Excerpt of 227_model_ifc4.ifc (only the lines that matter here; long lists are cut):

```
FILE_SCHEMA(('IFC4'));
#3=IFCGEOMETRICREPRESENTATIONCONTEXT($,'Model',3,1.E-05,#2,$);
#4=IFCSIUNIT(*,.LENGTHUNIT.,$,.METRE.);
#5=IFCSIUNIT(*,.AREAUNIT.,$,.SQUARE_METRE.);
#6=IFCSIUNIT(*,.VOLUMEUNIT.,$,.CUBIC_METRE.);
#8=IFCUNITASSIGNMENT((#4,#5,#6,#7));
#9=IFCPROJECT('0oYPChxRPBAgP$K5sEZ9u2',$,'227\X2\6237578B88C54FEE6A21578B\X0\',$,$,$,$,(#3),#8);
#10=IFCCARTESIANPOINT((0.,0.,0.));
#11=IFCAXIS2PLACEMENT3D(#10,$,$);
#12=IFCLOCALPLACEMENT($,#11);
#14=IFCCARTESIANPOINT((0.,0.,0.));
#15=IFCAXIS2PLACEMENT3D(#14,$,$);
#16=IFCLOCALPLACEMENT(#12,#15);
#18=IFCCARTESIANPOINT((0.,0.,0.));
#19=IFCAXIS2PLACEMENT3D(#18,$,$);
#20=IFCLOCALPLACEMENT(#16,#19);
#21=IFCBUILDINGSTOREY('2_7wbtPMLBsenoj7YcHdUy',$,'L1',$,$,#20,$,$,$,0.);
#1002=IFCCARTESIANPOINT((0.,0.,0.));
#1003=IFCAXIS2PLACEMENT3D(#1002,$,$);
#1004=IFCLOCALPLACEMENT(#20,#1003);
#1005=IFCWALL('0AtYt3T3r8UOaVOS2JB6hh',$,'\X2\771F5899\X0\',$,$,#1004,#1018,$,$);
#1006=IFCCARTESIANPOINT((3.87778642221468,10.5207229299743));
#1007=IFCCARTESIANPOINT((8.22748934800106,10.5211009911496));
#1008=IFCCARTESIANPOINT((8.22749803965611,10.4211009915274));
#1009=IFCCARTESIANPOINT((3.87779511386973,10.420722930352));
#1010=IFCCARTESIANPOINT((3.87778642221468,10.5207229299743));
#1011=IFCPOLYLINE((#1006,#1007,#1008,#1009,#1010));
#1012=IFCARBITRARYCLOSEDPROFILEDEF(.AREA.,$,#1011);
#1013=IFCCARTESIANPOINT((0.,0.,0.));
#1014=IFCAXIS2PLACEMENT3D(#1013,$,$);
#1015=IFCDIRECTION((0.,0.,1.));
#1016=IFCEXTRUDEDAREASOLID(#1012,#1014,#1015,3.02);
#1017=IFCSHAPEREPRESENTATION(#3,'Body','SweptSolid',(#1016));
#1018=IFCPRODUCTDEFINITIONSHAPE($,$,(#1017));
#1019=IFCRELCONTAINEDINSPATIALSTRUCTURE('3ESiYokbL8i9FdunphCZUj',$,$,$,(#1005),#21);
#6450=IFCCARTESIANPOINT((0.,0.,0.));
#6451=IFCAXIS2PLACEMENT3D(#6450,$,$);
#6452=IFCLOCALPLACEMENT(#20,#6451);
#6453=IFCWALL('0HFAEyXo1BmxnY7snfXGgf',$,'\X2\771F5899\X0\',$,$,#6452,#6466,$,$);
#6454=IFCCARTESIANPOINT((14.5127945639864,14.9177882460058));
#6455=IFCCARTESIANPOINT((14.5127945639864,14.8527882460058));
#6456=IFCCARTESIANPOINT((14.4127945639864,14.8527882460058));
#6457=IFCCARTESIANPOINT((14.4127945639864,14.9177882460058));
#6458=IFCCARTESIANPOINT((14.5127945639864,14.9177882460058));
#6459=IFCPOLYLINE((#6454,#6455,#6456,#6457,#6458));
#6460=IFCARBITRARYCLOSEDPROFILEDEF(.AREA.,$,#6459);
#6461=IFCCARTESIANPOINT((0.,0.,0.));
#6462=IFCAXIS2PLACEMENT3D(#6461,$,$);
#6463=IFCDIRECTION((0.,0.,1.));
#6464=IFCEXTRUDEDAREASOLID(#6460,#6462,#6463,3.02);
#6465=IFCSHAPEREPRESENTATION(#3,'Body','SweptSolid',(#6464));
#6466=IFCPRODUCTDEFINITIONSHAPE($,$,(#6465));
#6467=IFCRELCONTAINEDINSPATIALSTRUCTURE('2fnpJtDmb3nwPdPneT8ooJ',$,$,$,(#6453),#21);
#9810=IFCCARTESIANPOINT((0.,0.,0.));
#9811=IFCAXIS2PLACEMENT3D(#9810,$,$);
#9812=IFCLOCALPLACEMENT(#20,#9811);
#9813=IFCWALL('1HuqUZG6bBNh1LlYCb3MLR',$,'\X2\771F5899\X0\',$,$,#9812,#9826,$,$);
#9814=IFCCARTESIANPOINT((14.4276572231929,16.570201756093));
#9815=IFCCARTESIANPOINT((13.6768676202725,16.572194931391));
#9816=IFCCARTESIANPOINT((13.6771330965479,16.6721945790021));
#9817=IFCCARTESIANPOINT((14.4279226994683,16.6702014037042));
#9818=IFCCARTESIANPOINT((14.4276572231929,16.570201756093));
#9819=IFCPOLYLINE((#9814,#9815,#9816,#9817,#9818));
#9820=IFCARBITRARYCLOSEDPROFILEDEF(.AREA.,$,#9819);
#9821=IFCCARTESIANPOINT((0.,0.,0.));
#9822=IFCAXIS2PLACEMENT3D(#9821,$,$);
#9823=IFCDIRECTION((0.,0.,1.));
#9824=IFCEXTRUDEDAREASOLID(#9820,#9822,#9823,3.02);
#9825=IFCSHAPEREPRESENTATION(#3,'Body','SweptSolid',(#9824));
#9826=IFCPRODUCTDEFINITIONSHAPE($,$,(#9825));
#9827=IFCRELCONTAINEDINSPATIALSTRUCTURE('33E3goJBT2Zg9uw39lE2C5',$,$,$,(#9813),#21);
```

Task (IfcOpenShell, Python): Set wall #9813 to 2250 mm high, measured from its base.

```python
import ifcopenshell
import ifcopenshell.geom
import ifcopenshell.util.shape
import ifcopenshell.util.unit

model = ifcopenshell.open("227_model_ifc4.ifc")
unit_scale = ifcopenshell.util.unit.calculate_unit_scale(model)
settings = ifcopenshell.geom.settings()


def volume(element):
    """Net volume in cubic metres, openings subtracted."""
    shape = ifcopenshell.geom.create_shape(settings, element)
    return ifcopenshell.util.shape.get_volume(shape.geometry)


wall = model.by_guid("1HuqUZG6bBNh1LlYCb3MLR")
before = volume(wall)

body = next(r for r in wall.Representation.Representations if r.RepresentationIdentifier == "Body")
solid = body.Items[0]
old_height = solid.Depth
solid.Depth = 2.25 / unit_scale
after = volume(wall)

print(f"height {old_height:g} -> {solid.Depth:g}, volume {before:.3f} -> {after:.3f} m3")

model.write("227_model_ifc4-out.ifc")
```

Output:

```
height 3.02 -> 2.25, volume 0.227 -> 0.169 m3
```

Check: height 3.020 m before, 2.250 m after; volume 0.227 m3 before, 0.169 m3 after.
